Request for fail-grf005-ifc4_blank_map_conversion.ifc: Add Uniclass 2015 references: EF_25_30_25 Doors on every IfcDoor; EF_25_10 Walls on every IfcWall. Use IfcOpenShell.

First a look at what the model holds.

```python
import ifcopenshell

model = ifcopenshell.open("fail-grf005-ifc4_blank_map_conversion.ifc")
print(model.schema)
print("classifications:", [c.Name for c in model.by_type("IfcClassification")])
for ifc_class in ("IfcDoor", "IfcRoof", "IfcStair", "IfcWall", "IfcWindow"):
    print(ifc_class, len(model.by_type(ifc_class)))
```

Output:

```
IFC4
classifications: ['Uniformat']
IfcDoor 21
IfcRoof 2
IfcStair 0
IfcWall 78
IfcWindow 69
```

```python
import ifcopenshell
import ifcopenshell.api.classification

model = ifcopenshell.open("fail-grf005-ifc4_blank_map_conversion.ifc")

system = ifcopenshell.api.classification.add_classification(model, classification="Uniclass 2015")

codes = {
    "IfcDoor": ("EF_25_30_25", "Doors"),
    "IfcWall": ("EF_25_10", "Walls"),
}
for ifc_class, (code, name) in codes.items():
    products = model.by_type(ifc_class)
    ifcopenshell.api.classification.add_reference(
        model, products=products, classification=system, identification=code, name=name
    )
    print(code, len(products))

model.write("fail-grf005-ifc4_blank_map_conversion_edited.ifc")
```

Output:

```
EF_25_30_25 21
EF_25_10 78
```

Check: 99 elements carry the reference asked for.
